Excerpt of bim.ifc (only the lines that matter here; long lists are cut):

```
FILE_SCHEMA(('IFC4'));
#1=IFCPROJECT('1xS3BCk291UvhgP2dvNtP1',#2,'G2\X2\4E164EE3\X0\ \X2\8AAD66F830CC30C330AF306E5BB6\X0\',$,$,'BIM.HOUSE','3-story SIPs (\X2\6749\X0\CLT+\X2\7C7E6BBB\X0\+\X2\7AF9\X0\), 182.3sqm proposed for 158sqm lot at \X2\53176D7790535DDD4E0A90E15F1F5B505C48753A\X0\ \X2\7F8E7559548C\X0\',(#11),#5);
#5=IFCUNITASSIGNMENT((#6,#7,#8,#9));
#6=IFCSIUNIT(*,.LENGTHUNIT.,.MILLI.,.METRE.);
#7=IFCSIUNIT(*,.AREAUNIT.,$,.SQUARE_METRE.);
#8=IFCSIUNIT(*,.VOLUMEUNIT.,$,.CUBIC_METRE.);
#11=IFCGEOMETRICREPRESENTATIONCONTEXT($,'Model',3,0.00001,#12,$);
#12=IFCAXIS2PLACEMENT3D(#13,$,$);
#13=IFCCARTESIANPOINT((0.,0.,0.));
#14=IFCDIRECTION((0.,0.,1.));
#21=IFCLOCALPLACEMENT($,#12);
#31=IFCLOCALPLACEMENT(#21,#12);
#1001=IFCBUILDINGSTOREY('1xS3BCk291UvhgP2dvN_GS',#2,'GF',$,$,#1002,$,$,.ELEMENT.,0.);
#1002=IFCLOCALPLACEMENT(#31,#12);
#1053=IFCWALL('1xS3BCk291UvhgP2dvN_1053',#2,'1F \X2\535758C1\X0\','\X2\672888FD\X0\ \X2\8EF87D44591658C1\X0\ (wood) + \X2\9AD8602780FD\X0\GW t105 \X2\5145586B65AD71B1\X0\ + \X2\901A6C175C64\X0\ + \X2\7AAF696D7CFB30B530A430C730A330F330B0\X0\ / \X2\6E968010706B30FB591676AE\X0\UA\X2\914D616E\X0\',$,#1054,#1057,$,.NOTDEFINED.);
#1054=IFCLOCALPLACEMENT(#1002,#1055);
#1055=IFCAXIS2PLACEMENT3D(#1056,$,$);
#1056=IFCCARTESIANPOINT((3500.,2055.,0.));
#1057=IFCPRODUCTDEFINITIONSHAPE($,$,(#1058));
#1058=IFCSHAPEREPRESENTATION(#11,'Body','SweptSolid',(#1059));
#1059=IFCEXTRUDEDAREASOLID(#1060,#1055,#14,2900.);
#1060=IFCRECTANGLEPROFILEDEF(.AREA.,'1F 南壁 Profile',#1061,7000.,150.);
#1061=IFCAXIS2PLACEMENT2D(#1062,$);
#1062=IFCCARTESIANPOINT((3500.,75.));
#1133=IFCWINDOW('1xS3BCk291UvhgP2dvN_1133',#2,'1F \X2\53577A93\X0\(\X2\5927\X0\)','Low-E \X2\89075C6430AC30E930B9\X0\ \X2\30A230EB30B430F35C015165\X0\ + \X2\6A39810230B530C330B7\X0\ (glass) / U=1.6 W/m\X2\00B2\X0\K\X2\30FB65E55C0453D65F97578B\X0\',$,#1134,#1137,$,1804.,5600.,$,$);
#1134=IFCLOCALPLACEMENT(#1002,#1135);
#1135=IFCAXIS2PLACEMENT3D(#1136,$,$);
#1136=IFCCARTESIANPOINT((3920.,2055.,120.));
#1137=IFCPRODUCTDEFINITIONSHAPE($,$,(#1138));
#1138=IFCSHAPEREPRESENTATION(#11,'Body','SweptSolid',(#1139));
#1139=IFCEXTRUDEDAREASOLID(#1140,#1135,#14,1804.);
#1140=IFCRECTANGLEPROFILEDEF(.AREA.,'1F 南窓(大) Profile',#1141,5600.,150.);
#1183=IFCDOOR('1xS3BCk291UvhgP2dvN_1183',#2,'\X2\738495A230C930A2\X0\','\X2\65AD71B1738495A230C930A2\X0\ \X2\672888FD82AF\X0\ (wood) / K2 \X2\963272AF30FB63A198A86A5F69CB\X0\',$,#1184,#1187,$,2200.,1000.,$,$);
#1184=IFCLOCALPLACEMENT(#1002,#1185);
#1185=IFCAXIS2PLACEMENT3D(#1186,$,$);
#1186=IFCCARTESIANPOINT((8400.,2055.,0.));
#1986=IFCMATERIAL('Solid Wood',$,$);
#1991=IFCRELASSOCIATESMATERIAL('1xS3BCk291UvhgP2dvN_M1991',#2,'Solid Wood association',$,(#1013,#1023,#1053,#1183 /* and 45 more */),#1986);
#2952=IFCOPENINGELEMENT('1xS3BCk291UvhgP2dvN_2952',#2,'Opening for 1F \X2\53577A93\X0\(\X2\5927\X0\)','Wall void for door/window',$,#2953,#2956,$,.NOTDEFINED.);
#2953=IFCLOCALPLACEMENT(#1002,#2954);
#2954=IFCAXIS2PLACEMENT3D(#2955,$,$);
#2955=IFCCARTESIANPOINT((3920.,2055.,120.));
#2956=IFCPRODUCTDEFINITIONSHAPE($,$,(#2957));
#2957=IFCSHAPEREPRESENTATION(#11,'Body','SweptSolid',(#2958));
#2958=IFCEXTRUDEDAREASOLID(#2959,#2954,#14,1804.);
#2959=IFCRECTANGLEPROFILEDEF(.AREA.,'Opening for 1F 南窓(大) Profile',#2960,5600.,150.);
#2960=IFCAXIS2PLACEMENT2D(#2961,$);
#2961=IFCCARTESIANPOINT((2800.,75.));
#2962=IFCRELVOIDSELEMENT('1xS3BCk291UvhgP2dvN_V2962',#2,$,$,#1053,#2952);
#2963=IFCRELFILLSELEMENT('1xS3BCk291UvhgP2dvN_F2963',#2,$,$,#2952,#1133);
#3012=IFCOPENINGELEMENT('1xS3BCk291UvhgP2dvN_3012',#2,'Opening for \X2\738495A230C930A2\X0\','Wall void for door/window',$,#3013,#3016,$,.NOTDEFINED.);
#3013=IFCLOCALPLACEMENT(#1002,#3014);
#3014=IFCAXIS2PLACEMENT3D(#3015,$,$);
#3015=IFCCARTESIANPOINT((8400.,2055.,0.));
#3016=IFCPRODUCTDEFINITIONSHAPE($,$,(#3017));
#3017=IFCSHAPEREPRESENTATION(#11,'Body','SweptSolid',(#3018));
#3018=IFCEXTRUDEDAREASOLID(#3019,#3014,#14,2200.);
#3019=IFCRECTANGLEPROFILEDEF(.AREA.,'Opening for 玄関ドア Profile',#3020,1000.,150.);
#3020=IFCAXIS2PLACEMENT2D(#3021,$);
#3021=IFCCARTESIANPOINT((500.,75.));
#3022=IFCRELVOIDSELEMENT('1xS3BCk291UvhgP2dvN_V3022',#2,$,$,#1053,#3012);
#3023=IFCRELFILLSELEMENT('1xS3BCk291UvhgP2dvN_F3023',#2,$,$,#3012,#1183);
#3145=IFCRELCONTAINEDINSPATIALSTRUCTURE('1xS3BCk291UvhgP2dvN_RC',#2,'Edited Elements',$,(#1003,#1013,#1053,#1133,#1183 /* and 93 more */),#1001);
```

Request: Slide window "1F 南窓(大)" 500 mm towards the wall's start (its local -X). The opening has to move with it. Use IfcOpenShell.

```python
import ifcopenshell
import ifcopenshell.api.geometry
import ifcopenshell.util.placement

model = ifcopenshell.open("bim.ifc")

window = model.by_guid("1xS3BCk291UvhgP2dvN_1133")
opening = window.FillsVoids[0].RelatingOpeningElement
wall = opening.VoidsElements[0].RelatingBuildingElement

wall_matrix = ifcopenshell.util.placement.get_local_placement(wall.ObjectPlacement)
shift = wall_matrix[:3, 0] * -500.0
before = ifcopenshell.util.placement.get_local_placement(window.ObjectPlacement)[:3, 3].copy()

# The window is not placed relative to its opening, so move both.
for product in (opening, window):
    matrix = ifcopenshell.util.placement.get_local_placement(product.ObjectPlacement)
    matrix[:3, 3] += shift
    ifcopenshell.api.geometry.edit_object_placement(model, product=product, matrix=matrix, is_si=False)

after = ifcopenshell.util.placement.get_local_placement(window.ObjectPlacement)[:3, 3]
print("window moved by", (after - before).round(3) + 0.0)

model.write("bim_rev.ifc")
```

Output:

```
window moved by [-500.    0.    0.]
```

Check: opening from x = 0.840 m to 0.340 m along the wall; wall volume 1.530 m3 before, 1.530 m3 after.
